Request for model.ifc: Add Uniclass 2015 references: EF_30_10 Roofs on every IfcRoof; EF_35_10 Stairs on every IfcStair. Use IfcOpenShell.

First a look at what the model holds.

```python
import ifcopenshell

model = ifcopenshell.open("model.ifc")
print(model.schema)
print("classifications:", [c.Name for c in model.by_type("IfcClassification")])
for ifc_class in ("IfcDoor", "IfcRoof", "IfcStair", "IfcWall", "IfcWindow"):
    print(ifc_class, len(model.by_type(ifc_class)))
```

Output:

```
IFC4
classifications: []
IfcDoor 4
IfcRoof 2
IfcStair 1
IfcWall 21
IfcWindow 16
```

```python
import ifcopenshell
import ifcopenshell.api.classification

model = ifcopenshell.open("model.ifc")

system = ifcopenshell.api.classification.add_classification(model, classification="Uniclass 2015")

codes = {
    "IfcRoof": ("EF_30_10", "Roofs"),
    "IfcStair": ("EF_35_10", "Stairs"),
}
for ifc_class, (code, name) in codes.items():
    products = model.by_type(ifc_class)
    ifcopenshell.api.classification.add_reference(
        model, products=products, classification=system, identification=code, name=name
    )
    print(code, len(products))

model.write("model_rev.ifc")
```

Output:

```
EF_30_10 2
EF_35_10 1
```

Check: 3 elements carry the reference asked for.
